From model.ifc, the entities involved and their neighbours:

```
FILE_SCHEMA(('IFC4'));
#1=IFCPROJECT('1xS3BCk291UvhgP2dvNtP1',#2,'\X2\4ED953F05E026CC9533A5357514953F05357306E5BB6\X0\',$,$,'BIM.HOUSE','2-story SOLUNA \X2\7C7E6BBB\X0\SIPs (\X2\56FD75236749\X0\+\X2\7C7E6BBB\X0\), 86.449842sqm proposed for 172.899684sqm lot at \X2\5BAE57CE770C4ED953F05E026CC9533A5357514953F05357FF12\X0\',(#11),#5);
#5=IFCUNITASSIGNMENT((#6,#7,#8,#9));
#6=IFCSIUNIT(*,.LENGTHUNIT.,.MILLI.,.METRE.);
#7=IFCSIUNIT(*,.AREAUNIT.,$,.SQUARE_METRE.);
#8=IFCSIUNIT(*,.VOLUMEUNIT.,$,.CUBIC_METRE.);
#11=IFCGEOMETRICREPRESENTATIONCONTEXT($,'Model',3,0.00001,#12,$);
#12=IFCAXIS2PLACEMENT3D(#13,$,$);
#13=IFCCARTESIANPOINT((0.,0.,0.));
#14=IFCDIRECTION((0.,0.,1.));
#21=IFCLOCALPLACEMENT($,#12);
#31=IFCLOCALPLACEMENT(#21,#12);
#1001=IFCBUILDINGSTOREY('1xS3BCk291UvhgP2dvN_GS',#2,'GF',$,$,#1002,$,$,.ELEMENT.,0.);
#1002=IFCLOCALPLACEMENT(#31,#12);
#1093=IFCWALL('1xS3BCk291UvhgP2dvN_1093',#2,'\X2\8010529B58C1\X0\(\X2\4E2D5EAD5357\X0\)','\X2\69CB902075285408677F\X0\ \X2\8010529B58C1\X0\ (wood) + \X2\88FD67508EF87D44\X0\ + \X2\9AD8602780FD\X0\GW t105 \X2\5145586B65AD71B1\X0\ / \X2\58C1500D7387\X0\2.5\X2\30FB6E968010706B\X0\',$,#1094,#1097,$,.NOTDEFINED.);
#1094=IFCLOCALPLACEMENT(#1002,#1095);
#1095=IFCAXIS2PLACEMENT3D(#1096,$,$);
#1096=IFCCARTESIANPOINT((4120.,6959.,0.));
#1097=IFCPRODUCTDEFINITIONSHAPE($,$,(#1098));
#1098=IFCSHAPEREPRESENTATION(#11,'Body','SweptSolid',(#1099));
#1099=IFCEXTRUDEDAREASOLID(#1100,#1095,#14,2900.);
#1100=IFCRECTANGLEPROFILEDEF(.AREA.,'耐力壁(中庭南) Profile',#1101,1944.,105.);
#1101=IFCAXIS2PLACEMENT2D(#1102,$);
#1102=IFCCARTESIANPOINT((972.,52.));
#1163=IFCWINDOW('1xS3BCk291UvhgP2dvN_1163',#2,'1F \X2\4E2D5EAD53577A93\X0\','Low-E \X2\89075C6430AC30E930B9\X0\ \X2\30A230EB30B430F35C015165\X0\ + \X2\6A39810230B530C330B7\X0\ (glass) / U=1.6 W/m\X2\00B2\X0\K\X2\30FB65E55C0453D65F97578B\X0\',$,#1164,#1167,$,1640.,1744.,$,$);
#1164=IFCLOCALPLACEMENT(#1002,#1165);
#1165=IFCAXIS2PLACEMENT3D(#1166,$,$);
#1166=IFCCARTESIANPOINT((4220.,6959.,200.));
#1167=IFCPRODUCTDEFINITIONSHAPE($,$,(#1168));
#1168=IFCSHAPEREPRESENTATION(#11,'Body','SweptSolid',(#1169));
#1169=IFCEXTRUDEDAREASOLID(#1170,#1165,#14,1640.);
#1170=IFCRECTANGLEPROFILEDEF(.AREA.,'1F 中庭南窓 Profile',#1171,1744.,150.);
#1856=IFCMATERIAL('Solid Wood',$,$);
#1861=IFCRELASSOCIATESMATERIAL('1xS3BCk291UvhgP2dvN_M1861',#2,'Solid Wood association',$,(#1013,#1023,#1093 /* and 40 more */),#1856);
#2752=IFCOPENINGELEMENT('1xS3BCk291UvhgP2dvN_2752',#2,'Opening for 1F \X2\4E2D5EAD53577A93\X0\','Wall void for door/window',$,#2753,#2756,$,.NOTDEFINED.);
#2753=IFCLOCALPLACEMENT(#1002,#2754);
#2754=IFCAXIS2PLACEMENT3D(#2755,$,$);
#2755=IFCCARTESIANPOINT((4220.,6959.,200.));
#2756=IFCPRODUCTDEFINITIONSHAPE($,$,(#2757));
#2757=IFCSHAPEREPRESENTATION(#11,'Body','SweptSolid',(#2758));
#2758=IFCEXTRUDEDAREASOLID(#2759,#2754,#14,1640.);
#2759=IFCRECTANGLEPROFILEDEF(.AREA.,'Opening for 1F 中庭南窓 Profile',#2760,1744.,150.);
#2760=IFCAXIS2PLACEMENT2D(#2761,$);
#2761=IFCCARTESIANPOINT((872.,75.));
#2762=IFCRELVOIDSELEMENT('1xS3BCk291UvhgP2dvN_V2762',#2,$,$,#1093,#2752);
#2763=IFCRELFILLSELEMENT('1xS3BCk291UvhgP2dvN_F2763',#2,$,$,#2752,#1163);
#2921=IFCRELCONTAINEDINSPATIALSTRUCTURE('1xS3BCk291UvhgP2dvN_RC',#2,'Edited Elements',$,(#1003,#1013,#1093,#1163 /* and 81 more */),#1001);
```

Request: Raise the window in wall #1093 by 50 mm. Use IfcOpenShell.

```python
import numpy as np
import ifcopenshell
import ifcopenshell.api.geometry
import ifcopenshell.util.placement
import ifcopenshell.util.unit

model = ifcopenshell.open("model.ifc")
unit_scale = ifcopenshell.util.unit.calculate_unit_scale(model)

window = model.by_guid("1xS3BCk291UvhgP2dvN_1163")
opening = window.FillsVoids[0].RelatingOpeningElement
dz = 0.05 / unit_scale

shift = np.array([0.0, 0.0, dz])
# The window is not placed relative to its opening, so move both.
for product in (opening, window):
    matrix = ifcopenshell.util.placement.get_local_placement(product.ObjectPlacement)
    matrix[:3, 3] += shift
    ifcopenshell.api.geometry.edit_object_placement(model, product=product, matrix=matrix, is_si=False)

print(f"moved by {dz * unit_scale:+.3f} m")

model.write("model-out.ifc")
```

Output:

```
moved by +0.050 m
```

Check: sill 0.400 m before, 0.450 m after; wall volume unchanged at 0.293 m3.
